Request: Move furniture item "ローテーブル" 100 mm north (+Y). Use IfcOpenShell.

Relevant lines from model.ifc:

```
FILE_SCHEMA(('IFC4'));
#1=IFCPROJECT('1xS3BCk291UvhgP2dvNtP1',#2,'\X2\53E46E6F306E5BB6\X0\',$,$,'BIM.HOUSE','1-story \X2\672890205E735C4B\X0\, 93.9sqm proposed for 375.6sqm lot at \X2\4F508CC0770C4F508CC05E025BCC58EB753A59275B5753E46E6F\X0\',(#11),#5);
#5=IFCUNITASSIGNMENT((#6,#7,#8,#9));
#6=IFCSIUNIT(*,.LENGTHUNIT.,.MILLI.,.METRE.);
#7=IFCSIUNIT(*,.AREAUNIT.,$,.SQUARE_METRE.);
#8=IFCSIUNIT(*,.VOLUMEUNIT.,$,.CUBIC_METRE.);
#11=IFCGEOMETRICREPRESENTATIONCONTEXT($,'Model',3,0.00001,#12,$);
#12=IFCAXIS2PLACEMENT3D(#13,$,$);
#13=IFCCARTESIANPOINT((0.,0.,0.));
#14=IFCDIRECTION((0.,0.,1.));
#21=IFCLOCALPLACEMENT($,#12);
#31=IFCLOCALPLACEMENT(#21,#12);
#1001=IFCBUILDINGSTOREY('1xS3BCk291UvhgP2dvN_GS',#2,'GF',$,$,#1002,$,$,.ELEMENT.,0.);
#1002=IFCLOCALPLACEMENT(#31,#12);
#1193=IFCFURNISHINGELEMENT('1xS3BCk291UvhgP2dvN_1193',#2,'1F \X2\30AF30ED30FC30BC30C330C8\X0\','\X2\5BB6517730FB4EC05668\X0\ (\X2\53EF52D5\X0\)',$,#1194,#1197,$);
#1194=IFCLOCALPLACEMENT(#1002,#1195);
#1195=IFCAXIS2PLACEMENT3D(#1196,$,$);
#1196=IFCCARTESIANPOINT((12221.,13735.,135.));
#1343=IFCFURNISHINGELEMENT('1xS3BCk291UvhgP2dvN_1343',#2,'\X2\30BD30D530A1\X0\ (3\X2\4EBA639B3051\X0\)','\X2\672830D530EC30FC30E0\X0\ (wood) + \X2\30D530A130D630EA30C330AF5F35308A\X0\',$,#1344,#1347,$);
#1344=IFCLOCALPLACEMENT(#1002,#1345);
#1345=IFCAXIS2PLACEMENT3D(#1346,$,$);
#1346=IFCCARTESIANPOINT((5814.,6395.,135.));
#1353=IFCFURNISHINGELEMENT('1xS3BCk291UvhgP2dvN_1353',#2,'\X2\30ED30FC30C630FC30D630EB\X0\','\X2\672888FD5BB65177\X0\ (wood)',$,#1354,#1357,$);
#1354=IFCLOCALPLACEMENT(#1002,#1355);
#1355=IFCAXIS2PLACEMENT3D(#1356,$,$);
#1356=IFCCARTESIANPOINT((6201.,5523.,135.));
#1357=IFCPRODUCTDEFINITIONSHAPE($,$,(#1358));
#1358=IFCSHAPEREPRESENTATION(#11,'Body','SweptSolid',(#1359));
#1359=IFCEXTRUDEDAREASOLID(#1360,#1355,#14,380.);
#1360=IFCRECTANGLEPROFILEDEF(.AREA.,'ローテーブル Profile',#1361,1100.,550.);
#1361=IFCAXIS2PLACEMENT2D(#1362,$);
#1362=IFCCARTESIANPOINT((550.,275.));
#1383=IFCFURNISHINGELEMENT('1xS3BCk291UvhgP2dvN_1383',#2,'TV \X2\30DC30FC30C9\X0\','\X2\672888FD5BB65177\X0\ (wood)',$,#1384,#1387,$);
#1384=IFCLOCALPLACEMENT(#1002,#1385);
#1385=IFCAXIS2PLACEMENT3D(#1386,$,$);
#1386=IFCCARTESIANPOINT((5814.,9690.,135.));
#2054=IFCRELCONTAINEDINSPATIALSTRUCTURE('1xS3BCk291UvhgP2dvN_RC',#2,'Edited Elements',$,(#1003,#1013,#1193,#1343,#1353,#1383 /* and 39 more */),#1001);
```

```python
import ifcopenshell
import ifcopenshell.api.geometry
import ifcopenshell.util.placement

model = ifcopenshell.open("model.ifc")

item = model.by_id(1353)
matrix = ifcopenshell.util.placement.get_local_placement(item.ObjectPlacement)
matrix[1, 3] += 100.0
ifcopenshell.api.geometry.edit_object_placement(model, product=item, matrix=matrix, is_si=False)

print(ifcopenshell.util.placement.get_local_placement(item.ObjectPlacement).round(3) + 0.0)

model.write("model_edited.ifc")
```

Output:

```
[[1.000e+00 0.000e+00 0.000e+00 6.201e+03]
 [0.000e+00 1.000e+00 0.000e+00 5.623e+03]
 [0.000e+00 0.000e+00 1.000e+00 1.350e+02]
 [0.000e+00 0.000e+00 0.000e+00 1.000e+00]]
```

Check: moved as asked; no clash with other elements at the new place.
